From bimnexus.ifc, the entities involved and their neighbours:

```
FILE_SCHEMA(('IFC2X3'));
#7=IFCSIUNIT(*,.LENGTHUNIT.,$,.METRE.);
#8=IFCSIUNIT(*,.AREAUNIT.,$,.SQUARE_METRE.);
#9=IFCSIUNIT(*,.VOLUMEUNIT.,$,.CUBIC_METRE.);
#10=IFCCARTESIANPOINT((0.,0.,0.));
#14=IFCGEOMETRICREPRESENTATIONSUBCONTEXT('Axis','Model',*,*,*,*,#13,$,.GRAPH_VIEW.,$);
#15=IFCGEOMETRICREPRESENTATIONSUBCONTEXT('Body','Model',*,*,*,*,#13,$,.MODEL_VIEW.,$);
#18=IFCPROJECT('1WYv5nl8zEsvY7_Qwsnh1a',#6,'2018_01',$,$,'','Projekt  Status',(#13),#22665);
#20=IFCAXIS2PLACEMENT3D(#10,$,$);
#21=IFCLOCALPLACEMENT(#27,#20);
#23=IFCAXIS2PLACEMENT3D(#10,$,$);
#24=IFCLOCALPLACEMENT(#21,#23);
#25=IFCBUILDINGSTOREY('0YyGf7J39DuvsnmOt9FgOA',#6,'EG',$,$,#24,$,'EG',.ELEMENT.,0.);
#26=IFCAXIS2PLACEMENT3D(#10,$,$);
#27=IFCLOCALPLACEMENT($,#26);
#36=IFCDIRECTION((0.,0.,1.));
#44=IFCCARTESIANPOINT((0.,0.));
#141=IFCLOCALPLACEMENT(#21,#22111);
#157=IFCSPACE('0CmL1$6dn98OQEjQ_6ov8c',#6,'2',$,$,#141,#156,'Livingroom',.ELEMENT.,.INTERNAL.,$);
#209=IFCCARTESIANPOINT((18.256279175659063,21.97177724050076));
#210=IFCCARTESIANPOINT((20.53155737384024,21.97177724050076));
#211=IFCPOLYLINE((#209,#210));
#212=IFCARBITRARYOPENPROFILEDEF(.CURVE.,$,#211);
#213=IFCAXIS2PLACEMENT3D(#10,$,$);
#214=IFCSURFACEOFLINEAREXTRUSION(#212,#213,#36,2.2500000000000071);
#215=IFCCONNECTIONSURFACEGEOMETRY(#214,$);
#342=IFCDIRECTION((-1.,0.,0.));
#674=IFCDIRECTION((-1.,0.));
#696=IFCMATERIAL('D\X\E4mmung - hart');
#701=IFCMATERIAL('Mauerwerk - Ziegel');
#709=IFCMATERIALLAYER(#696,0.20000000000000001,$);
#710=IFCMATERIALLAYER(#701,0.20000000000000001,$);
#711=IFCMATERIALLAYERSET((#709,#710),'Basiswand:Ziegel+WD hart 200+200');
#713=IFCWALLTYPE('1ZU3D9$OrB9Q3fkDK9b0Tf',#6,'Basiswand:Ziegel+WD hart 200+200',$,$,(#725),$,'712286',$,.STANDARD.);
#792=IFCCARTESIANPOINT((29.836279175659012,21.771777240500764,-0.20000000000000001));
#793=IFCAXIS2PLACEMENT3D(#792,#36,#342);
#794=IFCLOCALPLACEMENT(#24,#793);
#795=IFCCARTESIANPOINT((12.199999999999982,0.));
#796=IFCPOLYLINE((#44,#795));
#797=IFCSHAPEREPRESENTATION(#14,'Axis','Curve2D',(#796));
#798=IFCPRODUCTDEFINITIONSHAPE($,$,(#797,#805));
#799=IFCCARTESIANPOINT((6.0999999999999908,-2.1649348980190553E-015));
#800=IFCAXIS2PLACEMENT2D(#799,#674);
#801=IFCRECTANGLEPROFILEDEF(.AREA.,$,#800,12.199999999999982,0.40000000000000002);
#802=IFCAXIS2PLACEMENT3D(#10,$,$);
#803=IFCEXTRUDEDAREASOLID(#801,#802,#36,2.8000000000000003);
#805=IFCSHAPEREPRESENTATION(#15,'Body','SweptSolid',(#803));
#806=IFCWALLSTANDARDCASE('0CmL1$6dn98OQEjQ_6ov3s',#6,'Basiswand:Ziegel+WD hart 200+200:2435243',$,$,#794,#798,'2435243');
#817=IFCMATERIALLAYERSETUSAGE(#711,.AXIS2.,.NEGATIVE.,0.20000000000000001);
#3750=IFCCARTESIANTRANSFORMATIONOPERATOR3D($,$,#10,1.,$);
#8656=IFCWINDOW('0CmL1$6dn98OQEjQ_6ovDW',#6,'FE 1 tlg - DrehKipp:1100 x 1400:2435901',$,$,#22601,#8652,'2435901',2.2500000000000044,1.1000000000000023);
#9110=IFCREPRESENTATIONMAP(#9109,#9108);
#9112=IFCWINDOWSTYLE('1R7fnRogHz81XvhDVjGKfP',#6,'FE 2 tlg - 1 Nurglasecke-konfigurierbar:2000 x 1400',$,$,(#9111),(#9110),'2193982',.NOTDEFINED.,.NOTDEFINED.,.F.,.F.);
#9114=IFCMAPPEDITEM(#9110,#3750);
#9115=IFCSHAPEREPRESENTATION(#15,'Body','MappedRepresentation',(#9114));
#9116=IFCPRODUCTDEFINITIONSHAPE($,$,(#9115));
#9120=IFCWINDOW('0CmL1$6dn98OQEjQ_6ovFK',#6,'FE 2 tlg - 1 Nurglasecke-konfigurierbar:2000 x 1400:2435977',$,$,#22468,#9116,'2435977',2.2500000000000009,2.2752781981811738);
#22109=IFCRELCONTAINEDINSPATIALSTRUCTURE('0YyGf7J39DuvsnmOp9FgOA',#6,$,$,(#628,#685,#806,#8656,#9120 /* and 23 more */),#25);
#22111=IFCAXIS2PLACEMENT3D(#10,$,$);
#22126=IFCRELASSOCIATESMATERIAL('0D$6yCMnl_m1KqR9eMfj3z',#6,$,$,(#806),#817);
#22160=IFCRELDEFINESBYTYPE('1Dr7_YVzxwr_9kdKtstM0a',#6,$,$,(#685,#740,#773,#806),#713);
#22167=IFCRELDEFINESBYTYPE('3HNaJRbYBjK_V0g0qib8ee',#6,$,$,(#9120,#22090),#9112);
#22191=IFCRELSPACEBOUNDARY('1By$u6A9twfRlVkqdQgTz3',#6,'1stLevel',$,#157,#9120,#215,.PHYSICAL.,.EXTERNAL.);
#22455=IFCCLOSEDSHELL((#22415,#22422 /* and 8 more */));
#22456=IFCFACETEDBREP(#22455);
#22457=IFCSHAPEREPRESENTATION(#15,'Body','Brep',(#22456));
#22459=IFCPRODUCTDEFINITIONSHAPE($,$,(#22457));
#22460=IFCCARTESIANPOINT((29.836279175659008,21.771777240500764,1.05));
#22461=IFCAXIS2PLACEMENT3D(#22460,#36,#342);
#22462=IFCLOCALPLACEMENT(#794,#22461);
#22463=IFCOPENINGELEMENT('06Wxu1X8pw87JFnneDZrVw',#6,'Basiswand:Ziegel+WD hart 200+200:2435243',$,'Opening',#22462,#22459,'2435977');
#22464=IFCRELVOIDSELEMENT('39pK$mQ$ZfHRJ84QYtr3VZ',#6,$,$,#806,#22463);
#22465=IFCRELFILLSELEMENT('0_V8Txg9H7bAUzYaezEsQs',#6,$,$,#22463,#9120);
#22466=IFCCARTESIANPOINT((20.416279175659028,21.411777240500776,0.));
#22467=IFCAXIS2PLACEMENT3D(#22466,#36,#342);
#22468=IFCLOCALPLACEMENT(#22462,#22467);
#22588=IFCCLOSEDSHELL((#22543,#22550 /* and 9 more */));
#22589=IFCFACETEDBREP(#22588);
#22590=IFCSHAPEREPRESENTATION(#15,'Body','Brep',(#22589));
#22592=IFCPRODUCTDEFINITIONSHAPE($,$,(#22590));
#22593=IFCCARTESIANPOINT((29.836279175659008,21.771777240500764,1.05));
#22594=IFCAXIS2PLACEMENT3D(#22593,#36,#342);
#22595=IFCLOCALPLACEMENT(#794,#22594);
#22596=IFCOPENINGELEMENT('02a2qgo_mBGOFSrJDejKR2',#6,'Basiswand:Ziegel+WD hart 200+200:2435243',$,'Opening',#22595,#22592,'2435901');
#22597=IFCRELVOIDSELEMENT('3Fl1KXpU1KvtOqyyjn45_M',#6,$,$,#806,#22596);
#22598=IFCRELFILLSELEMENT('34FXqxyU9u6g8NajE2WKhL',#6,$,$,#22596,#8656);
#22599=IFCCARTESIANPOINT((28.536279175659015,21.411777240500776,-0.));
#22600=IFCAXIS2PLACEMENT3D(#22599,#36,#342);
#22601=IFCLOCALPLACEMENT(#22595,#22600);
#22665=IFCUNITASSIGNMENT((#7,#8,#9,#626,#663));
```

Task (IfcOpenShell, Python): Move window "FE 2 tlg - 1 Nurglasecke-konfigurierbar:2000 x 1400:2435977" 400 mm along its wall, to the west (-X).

```python
import numpy as np
import ifcopenshell
import ifcopenshell.api.geometry
import ifcopenshell.util.placement
import ifcopenshell.util.unit

model = ifcopenshell.open("bimnexus.ifc")
unit_scale = ifcopenshell.util.unit.calculate_unit_scale(model)

window = model.by_guid("0CmL1$6dn98OQEjQ_6ovFK")
opening = window.FillsVoids[0].RelatingOpeningElement
wall = opening.VoidsElements[0].RelatingBuildingElement

wall_matrix = ifcopenshell.util.placement.get_local_placement(wall.ObjectPlacement)
shift = wall_matrix[:3, 0] * 0.4 / unit_scale
before = ifcopenshell.util.placement.get_local_placement(window.ObjectPlacement)[:3, 3].copy()

# The window is placed relative to its opening, so it follows when the opening moves.
matrix = ifcopenshell.util.placement.get_local_placement(opening.ObjectPlacement)
matrix[:3, 3] += shift
ifcopenshell.api.geometry.edit_object_placement(
    model, product=opening, matrix=matrix, is_si=False, should_transform_children=True
)

# Space boundary surfaces are stored in each space's coordinates; move them too.
for rel in window.ProvidesBoundaries:
    if not rel.ConnectionGeometry:
        continue
    surface = rel.ConnectionGeometry.SurfaceOnRelatingElement
    space_matrix = ifcopenshell.util.placement.get_local_placement(rel.RelatingSpace.ObjectPlacement)
    point = np.array(surface.Position.Location.Coordinates) + space_matrix[:3, :3].T @ shift
    surface.Position = model.createIfcAxis2Placement3D(
        model.createIfcCartesianPoint(point.tolist()), surface.Position.Axis, surface.Position.RefDirection
    )

after = ifcopenshell.util.placement.get_local_placement(window.ObjectPlacement)[:3, 3]
print("window moved by", (after - before).round(3) + 0.0)

model.write("bimnexus_edited.ifc")
```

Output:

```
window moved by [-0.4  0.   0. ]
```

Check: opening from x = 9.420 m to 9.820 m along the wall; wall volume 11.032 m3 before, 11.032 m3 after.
